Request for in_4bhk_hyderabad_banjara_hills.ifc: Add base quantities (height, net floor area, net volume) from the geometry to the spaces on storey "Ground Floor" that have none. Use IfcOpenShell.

First a look at what the model holds.

```python
import ifcopenshell
import ifcopenshell.util.element
import ifcopenshell.util.unit

model = ifcopenshell.open("in_4bhk_hyderabad_banjara_hills.ifc")
print(model.schema)
for unit_type in ("LENGTHUNIT", "AREAUNIT", "VOLUMEUNIT"):
    print(unit_type, ifcopenshell.util.unit.calculate_unit_scale(model, unit_type))
storey = next(s for s in model.by_type("IfcBuildingStorey") if s.Name == "Ground Floor")
spaces = [e for e in ifcopenshell.util.element.get_decomposition(storey) if e.is_a("IfcSpace")]
for e in sorted(spaces, key=lambda e: e.id()):
    print(e.id(), e.is_a(), e.Name, list(ifcopenshell.util.element.get_psets(e, qtos_only=True)), sep=" | ")
```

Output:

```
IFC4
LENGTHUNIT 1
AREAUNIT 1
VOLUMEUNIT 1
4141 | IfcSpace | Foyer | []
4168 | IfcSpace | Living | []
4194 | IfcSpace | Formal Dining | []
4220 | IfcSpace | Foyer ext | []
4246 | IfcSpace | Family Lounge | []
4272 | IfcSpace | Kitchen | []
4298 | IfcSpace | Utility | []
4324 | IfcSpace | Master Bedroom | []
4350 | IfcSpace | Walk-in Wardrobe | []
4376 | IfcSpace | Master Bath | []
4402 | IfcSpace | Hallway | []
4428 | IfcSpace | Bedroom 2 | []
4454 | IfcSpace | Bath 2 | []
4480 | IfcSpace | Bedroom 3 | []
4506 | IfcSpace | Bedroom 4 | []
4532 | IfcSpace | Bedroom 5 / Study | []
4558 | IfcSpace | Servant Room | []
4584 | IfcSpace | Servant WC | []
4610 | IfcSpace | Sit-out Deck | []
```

```python
import ifcopenshell
import ifcopenshell.api.pset
import ifcopenshell.geom
import ifcopenshell.util.element
import ifcopenshell.util.shape
import ifcopenshell.util.unit

model = ifcopenshell.open("in_4bhk_hyderabad_banjara_hills.ifc")
unit_scale = ifcopenshell.util.unit.calculate_unit_scale(model)
area_scale = ifcopenshell.util.unit.calculate_unit_scale(model, "AREAUNIT")
volume_scale = ifcopenshell.util.unit.calculate_unit_scale(model, "VOLUMEUNIT")
settings = ifcopenshell.geom.settings()

storey = next(s for s in model.by_type("IfcBuildingStorey") if s.Name == "Ground Floor")
spaces = [e for e in ifcopenshell.util.element.get_decomposition(storey) if e.is_a("IfcSpace")]

for e in sorted(spaces, key=lambda e: e.id()):
    if ifcopenshell.util.element.get_psets(e, qtos_only=True, should_inherit=False):
        continue
    # Geometry comes back in metres, in the element's own axes.
    shape = ifcopenshell.geom.create_shape(settings, e)
    values = {
        "Height": ifcopenshell.util.shape.get_z(shape.geometry) / unit_scale,
        "NetFloorArea": ifcopenshell.util.shape.get_footprint_area(shape.geometry) / area_scale,
        "NetVolume": ifcopenshell.util.shape.get_volume(shape.geometry) / volume_scale,
    }
    qto = ifcopenshell.api.pset.add_qto(model, product=e, name="Qto_SpaceBaseQuantities")
    ifcopenshell.api.pset.edit_qto(model, qto=qto, properties=values)
    print(e.id(), {k: round(v, 3) for k, v in values.items()})

model.write("in_4bhk_hyderabad_banjara_hills_v2.ifc")
```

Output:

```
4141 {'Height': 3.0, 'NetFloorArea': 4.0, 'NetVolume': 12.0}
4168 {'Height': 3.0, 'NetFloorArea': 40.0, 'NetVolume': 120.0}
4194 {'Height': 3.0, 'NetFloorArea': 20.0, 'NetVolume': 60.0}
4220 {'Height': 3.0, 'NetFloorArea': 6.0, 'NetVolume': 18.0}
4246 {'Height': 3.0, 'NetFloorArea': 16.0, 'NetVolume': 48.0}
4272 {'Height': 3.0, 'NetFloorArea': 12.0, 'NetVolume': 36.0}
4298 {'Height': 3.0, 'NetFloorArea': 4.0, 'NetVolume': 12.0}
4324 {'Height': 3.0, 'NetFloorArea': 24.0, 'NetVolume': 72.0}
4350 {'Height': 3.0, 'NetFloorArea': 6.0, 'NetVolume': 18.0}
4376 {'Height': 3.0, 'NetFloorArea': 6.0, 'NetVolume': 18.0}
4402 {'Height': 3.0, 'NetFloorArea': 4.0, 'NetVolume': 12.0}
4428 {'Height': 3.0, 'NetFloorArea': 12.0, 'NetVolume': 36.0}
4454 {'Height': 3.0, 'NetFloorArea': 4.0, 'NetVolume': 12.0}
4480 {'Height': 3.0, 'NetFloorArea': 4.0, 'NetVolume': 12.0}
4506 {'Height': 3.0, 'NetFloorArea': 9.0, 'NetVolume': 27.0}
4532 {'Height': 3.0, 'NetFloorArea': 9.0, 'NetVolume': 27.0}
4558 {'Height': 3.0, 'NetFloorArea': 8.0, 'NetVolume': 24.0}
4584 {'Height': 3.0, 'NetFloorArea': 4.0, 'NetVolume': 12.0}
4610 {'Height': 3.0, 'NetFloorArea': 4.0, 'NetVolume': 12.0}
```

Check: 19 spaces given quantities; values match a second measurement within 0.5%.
